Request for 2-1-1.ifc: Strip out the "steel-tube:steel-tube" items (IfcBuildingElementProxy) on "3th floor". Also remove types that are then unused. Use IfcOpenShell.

First a look at what the model holds.

```python
import ifcopenshell
import ifcopenshell.util.element

model = ifcopenshell.open("2-1-1.ifc")
print(model.schema)
storey = next(s for s in model.by_type("IfcBuildingStorey") if s.Name == "3th floor")
proxies = [e for e in ifcopenshell.util.element.get_decomposition(storey) if e.is_a("IfcBuildingElementProxy")]
seen = {}
for e in proxies:
    element_type = ifcopenshell.util.element.get_type(e)
    name = element_type.Name if element_type not in (None, e) else None
    seen[name] = seen.get(name, 0) + 1
for name, count in sorted(seen.items(), key=str):
    print(count, "x", name)
```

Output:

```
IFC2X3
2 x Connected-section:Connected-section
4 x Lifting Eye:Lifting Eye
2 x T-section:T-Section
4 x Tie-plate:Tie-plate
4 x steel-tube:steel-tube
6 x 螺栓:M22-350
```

```python
import ifcopenshell
import ifcopenshell.api.root
import ifcopenshell.util.element

model = ifcopenshell.open("2-1-1.ifc")

storey = next(s for s in model.by_type("IfcBuildingStorey") if s.Name == "3th floor")
proxies = [e for e in ifcopenshell.util.element.get_decomposition(storey) if e.is_a("IfcBuildingElementProxy")]
targets = [e for e in proxies if (t := ifcopenshell.util.element.get_type(e)) not in (None, e) and t.Name == "steel-tube:steel-tube"]
types = {ifcopenshell.util.element.get_type(e) for e in targets} - {None, *targets}

for e in targets:
    ifcopenshell.api.root.remove_product(model, product=e)
print(len(targets), "removed")

unused = [t for t in types if not ifcopenshell.util.element.get_types(t)]
for t in unused:
    ifcopenshell.api.root.remove_product(model, product=t)
print(len(unused), "unused types removed")

model.write("2-1-1-out.ifc")
```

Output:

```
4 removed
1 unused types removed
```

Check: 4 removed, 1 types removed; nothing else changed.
